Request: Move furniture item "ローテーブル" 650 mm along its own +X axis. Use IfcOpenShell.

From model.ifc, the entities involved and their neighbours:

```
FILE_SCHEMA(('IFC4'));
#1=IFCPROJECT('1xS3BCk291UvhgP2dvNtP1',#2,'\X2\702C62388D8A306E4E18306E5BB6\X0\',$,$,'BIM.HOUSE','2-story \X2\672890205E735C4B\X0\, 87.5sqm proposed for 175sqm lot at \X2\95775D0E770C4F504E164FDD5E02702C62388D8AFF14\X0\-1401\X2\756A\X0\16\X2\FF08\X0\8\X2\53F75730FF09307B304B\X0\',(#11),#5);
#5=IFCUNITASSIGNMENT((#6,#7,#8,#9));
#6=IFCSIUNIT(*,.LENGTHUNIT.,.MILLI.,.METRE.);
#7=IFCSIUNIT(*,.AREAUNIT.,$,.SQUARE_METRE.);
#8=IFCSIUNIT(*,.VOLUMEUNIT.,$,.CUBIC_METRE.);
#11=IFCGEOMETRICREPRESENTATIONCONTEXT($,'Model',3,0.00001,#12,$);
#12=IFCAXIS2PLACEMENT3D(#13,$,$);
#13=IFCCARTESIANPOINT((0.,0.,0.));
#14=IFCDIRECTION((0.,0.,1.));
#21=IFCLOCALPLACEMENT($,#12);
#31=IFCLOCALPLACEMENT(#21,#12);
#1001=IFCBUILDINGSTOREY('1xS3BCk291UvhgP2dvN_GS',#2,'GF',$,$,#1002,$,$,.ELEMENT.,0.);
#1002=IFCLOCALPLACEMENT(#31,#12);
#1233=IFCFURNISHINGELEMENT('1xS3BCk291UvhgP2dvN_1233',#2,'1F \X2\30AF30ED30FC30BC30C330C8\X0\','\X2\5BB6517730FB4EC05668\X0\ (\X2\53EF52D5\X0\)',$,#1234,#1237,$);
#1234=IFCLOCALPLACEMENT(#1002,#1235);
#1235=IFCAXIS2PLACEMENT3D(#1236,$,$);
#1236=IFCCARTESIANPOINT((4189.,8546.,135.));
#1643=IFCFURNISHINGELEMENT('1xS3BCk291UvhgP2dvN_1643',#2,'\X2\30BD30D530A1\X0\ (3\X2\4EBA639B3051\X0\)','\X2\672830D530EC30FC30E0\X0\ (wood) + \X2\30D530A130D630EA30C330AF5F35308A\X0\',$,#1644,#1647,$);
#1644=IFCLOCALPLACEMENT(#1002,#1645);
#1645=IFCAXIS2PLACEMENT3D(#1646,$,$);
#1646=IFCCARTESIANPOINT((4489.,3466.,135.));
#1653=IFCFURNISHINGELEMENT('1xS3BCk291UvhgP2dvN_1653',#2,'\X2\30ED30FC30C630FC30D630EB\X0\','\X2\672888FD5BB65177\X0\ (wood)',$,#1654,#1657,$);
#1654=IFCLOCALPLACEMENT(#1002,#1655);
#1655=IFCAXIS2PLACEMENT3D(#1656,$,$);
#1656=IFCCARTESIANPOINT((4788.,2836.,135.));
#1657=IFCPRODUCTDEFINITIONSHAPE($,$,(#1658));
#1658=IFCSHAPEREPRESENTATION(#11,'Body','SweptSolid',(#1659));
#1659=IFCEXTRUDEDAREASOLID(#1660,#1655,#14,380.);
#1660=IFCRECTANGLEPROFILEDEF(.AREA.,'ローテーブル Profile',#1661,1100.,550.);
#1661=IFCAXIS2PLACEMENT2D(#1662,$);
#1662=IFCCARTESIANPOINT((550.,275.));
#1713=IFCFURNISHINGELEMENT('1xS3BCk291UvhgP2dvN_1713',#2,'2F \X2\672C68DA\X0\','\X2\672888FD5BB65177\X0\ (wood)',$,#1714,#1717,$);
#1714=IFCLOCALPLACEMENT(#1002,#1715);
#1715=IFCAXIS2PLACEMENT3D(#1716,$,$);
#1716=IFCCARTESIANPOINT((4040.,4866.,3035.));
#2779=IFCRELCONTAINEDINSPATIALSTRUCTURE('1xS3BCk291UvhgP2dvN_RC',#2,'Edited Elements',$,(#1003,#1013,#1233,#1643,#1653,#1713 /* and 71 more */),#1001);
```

```python
import ifcopenshell
import ifcopenshell.api.geometry
import ifcopenshell.util.placement
import ifcopenshell.util.unit

model = ifcopenshell.open("model.ifc")
unit_scale = ifcopenshell.util.unit.calculate_unit_scale(model)

item = model.by_guid("1xS3BCk291UvhgP2dvN_1653")
matrix = ifcopenshell.util.placement.get_local_placement(item.ObjectPlacement)
matrix[:3, 3] += matrix[:3, 0] * 0.65 / unit_scale
ifcopenshell.api.geometry.edit_object_placement(model, product=item, matrix=matrix, is_si=False)

print(ifcopenshell.util.placement.get_local_placement(item.ObjectPlacement).round(3) + 0.0)

model.write("model_v2.ifc")
```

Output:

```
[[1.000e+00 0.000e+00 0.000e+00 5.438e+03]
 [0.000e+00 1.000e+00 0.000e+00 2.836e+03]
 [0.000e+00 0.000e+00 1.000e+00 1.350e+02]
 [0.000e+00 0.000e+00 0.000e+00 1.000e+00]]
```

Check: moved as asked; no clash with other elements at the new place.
